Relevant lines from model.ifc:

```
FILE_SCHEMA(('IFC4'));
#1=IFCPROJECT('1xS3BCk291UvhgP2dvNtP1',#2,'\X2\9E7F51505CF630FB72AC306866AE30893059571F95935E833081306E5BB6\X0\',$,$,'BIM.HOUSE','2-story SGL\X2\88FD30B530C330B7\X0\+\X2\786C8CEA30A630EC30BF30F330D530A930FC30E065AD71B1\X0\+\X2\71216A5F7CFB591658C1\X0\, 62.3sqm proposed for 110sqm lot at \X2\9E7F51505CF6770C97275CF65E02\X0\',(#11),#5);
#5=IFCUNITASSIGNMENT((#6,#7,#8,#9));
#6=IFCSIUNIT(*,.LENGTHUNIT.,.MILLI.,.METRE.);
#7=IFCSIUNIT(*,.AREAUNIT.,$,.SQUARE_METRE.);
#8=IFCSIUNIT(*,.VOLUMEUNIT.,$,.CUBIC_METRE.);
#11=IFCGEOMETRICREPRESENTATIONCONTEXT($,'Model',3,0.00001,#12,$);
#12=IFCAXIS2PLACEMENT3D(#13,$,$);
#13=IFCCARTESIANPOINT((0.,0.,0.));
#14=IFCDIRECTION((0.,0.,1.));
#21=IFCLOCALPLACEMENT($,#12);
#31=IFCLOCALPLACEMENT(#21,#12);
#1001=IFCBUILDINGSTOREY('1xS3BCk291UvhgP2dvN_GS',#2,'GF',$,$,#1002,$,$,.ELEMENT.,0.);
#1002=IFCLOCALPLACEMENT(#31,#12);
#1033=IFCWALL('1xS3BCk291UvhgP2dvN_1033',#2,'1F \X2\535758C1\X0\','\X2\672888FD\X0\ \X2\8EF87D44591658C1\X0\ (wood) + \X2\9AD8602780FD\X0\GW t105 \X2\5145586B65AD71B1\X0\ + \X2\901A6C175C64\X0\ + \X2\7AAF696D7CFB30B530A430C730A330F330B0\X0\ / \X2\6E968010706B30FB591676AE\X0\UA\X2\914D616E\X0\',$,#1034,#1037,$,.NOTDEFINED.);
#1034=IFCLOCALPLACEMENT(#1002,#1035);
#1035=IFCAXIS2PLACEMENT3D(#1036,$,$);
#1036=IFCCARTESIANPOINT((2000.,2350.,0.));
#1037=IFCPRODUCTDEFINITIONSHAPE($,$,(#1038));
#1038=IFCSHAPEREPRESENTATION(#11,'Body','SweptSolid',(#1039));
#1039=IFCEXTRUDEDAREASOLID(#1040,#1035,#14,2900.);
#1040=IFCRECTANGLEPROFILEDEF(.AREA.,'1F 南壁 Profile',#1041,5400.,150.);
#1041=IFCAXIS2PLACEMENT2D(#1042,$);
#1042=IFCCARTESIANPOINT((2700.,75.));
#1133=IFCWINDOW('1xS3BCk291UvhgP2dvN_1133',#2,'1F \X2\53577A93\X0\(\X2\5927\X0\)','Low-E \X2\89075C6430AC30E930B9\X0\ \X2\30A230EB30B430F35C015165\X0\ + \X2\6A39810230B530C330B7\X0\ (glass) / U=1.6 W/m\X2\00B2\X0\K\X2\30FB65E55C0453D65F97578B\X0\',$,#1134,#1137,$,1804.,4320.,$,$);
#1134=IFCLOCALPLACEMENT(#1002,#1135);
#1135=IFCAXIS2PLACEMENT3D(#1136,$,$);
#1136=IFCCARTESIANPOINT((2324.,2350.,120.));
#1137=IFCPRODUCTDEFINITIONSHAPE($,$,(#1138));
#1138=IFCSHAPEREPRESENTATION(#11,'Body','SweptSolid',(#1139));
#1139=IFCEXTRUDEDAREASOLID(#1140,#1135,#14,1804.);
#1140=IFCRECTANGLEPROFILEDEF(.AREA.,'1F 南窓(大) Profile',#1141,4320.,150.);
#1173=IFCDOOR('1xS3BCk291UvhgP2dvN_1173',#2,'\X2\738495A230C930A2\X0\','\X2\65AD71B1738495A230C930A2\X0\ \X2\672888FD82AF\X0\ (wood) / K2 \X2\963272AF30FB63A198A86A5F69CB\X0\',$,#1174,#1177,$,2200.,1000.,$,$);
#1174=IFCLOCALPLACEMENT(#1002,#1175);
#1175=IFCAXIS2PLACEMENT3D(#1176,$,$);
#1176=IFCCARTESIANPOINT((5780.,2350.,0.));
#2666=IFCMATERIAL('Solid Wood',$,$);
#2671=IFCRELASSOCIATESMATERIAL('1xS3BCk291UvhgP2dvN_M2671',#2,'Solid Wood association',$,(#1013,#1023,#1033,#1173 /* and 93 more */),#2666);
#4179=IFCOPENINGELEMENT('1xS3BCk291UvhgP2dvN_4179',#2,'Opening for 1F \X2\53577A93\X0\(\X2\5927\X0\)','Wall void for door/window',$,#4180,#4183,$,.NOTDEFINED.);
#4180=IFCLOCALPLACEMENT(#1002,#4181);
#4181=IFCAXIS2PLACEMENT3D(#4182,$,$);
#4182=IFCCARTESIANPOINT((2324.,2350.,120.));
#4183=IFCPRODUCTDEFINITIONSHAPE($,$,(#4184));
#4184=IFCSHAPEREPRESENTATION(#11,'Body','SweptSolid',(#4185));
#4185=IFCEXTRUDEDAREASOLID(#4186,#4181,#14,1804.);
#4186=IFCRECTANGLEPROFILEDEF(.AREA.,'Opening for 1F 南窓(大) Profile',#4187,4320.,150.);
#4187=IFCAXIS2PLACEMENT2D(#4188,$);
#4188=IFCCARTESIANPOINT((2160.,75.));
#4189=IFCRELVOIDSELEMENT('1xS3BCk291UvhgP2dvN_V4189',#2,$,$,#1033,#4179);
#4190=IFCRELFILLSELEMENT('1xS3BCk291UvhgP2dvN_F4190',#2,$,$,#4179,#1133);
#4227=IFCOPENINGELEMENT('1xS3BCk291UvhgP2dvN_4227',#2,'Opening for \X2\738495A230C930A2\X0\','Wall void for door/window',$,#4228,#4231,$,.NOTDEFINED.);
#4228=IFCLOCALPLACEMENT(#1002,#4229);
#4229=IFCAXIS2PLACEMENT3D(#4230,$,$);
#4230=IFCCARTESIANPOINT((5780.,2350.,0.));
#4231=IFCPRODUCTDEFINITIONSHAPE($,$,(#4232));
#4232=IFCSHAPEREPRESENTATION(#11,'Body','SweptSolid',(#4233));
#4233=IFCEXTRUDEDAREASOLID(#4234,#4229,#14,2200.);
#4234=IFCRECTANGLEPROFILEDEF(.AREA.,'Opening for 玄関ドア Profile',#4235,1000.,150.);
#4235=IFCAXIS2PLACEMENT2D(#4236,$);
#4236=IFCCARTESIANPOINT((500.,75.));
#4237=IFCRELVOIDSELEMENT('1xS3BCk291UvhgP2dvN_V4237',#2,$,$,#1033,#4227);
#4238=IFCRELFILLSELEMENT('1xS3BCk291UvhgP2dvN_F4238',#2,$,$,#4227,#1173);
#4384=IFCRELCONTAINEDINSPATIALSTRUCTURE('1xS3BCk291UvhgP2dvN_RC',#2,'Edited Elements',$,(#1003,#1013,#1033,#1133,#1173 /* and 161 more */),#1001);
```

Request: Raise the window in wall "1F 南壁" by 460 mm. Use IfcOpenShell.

```python
import numpy as np
import ifcopenshell
import ifcopenshell.api.geometry
import ifcopenshell.util.placement
import ifcopenshell.util.unit

model = ifcopenshell.open("model.ifc")
unit_scale = ifcopenshell.util.unit.calculate_unit_scale(model)

window = model.by_id(1133)
opening = window.FillsVoids[0].RelatingOpeningElement
dz = 460.0

shift = np.array([0.0, 0.0, dz])
# The window is not placed relative to its opening, so move both.
for product in (opening, window):
    matrix = ifcopenshell.util.placement.get_local_placement(product.ObjectPlacement)
    matrix[:3, 3] += shift
    ifcopenshell.api.geometry.edit_object_placement(model, product=product, matrix=matrix, is_si=False)

print(f"moved by {dz * unit_scale:+.3f} m")

model.write("model_updated.ifc")
```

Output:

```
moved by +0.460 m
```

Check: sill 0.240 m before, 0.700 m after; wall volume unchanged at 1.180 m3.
